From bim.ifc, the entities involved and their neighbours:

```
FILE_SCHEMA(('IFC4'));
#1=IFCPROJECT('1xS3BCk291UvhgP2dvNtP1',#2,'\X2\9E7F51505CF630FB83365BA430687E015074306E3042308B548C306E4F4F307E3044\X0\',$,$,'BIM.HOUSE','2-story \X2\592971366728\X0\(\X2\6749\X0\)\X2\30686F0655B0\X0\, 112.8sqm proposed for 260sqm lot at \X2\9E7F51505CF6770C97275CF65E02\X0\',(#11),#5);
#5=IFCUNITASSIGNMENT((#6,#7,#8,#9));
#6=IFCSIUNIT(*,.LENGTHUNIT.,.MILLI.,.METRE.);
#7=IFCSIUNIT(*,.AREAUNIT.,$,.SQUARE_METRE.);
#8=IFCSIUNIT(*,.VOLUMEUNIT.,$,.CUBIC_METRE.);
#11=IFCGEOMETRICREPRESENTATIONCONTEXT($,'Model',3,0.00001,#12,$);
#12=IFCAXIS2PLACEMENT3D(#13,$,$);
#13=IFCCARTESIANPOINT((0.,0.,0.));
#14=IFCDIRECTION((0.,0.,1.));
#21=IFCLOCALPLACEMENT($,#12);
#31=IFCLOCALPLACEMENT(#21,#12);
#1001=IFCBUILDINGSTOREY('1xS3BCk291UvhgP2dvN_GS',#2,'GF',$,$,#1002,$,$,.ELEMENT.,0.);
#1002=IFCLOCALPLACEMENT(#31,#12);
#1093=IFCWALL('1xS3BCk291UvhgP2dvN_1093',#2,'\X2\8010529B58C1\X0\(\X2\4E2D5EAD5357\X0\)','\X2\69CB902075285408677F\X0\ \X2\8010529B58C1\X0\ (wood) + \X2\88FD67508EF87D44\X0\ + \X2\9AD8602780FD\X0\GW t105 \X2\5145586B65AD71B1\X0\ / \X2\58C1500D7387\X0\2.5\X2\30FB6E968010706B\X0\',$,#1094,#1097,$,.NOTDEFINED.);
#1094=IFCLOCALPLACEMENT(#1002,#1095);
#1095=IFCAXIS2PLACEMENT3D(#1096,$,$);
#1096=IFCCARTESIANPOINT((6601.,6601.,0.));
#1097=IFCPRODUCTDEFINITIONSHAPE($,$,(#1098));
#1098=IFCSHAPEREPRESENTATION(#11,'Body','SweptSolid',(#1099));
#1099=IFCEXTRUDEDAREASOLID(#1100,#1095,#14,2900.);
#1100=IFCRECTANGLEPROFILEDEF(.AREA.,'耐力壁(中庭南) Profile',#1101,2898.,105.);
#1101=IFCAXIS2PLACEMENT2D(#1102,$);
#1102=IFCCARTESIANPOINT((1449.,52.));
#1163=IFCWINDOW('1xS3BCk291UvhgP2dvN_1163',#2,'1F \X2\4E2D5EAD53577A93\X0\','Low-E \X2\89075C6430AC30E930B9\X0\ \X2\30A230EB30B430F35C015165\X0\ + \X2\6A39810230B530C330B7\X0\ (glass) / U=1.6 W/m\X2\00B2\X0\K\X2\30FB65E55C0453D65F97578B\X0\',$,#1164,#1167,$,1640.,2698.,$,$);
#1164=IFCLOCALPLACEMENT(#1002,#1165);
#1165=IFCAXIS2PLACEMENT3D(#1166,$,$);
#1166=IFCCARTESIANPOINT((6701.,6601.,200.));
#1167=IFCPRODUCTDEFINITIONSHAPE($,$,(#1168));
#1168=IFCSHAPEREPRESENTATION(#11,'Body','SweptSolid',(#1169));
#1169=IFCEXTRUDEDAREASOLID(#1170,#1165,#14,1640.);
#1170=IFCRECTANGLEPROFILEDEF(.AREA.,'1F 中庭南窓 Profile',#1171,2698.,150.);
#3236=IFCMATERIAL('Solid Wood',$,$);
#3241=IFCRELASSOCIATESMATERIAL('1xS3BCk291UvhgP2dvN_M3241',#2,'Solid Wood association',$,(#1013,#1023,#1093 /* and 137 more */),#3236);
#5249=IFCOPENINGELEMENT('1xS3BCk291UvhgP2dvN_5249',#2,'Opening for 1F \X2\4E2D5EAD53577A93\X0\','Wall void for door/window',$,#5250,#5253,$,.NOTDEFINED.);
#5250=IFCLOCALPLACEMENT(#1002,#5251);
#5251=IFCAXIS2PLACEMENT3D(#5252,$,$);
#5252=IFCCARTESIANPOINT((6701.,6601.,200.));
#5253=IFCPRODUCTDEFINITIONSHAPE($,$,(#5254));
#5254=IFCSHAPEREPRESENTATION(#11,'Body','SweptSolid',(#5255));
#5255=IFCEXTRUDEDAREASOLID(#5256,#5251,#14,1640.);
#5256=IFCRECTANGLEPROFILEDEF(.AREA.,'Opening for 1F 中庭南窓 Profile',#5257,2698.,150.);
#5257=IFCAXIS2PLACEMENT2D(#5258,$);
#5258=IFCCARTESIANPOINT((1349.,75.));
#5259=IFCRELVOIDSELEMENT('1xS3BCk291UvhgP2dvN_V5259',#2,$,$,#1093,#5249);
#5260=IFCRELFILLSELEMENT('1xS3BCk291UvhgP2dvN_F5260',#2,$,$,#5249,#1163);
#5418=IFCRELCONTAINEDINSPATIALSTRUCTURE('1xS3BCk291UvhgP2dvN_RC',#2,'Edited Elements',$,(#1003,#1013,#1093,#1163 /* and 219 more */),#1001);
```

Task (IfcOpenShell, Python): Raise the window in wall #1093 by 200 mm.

```python
import numpy as np
import ifcopenshell
import ifcopenshell.api.geometry
import ifcopenshell.util.placement
import ifcopenshell.util.unit

model = ifcopenshell.open("bim.ifc")
unit_scale = ifcopenshell.util.unit.calculate_unit_scale(model)

window = model.by_id(1163)
opening = window.FillsVoids[0].RelatingOpeningElement
dz = 200.0

shift = np.array([0.0, 0.0, dz])
# The window is not placed relative to its opening, so move both.
for product in (opening, window):
    matrix = ifcopenshell.util.placement.get_local_placement(product.ObjectPlacement)
    matrix[:3, 3] += shift
    ifcopenshell.api.geometry.edit_object_placement(model, product=product, matrix=matrix, is_si=False)

print(f"moved by {dz * unit_scale:+.3f} m")

model.write("bim_v2.ifc")
```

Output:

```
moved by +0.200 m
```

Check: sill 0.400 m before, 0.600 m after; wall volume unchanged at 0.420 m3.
